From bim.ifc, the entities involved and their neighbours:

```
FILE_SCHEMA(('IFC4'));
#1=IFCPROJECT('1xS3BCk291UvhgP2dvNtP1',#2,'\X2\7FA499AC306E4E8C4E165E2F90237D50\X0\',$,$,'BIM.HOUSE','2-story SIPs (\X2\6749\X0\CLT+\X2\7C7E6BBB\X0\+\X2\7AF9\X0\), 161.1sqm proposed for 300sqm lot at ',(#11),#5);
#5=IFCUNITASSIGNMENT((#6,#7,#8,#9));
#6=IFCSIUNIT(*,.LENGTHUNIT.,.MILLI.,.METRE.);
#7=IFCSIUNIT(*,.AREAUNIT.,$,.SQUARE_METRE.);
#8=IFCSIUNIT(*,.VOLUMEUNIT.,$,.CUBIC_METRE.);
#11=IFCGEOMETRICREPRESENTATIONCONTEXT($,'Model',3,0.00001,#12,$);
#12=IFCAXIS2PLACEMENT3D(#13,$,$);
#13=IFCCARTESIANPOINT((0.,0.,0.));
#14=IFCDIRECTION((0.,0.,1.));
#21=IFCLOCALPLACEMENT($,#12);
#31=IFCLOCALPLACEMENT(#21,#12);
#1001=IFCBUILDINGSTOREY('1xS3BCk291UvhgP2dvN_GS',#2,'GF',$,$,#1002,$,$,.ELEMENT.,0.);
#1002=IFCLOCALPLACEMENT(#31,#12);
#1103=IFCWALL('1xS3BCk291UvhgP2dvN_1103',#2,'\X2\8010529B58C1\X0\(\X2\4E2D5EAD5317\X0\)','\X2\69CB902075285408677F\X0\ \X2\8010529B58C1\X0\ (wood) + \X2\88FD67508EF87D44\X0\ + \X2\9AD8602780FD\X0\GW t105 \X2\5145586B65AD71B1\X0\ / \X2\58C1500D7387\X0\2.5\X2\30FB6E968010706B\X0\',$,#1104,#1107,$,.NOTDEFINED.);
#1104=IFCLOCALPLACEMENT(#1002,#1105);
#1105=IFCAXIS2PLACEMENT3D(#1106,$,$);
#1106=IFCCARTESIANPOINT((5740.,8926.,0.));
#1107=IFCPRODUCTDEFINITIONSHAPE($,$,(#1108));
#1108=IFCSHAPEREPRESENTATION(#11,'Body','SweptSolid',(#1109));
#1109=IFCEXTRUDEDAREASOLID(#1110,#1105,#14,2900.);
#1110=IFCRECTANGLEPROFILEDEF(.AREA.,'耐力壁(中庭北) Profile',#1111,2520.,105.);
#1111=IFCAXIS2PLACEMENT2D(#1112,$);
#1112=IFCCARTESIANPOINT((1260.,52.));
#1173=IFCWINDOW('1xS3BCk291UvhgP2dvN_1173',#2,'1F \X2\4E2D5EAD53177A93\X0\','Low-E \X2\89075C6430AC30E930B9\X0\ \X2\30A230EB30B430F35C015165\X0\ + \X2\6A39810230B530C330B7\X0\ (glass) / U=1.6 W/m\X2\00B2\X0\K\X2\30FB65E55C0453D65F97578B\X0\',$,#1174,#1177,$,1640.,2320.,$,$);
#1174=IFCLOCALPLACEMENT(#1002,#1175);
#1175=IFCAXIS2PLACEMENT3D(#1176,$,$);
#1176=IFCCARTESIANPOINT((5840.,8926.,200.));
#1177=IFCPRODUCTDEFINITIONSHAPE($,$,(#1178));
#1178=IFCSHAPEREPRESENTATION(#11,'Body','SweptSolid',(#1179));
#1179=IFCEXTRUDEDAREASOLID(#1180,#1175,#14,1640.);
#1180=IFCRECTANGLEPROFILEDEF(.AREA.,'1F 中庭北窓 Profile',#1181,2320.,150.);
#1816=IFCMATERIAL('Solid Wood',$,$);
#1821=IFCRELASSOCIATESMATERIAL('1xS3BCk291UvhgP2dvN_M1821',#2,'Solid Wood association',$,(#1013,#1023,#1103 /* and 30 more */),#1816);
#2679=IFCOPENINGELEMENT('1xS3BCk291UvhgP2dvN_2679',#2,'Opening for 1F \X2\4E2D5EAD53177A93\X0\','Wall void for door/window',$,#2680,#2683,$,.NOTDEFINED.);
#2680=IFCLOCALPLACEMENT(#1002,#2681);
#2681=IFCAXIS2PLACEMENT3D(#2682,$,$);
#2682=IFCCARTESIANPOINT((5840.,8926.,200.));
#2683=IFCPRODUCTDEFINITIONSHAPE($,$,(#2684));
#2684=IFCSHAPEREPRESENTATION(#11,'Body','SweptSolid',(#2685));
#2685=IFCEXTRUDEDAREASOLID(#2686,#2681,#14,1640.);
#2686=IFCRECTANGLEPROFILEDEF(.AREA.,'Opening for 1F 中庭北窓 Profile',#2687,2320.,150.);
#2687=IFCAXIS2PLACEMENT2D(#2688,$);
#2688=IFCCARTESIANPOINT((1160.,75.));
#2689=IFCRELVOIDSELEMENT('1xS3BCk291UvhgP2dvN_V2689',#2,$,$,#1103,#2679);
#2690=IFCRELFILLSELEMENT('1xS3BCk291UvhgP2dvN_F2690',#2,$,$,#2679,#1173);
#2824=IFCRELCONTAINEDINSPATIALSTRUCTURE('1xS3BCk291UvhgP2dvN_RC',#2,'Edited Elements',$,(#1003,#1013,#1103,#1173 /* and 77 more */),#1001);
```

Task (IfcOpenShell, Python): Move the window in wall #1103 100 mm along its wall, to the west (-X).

```python
import ifcopenshell
import ifcopenshell.api.geometry
import ifcopenshell.util.placement

model = ifcopenshell.open("bim.ifc")

window = model.by_guid("1xS3BCk291UvhgP2dvN_1173")
opening = window.FillsVoids[0].RelatingOpeningElement
wall = opening.VoidsElements[0].RelatingBuildingElement

wall_matrix = ifcopenshell.util.placement.get_local_placement(wall.ObjectPlacement)
shift = wall_matrix[:3, 0] * -100.0
before = ifcopenshell.util.placement.get_local_placement(window.ObjectPlacement)[:3, 3].copy()

# The window is not placed relative to its opening, so move both.
for product in (opening, window):
    matrix = ifcopenshell.util.placement.get_local_placement(product.ObjectPlacement)
    matrix[:3, 3] += shift
    ifcopenshell.api.geometry.edit_object_placement(model, product=product, matrix=matrix, is_si=False)

after = ifcopenshell.util.placement.get_local_placement(window.ObjectPlacement)[:3, 3]
print("window moved by", (after - before).round(3) + 0.0)

model.write("bim_rev.ifc")
```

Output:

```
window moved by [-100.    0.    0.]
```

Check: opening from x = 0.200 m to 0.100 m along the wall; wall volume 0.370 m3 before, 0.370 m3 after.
